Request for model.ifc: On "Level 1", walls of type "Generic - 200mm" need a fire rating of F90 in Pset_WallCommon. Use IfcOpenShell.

First a look at what the model holds.

```python
import ifcopenshell
import ifcopenshell.util.element

model = ifcopenshell.open("model.ifc")
print(model.schema)
storey = next(s for s in model.by_type("IfcBuildingStorey") if s.Name == "Level 1")
walls = [e for e in ifcopenshell.util.element.get_decomposition(storey) if e.is_a("IfcWall")]
seen = {}
for e in walls:
    element_type = ifcopenshell.util.element.get_type(e)
    key = (element_type.Name if element_type != e and element_type else None, ifcopenshell.util.element.get_pset(e, "Pset_WallCommon", "FireRating"))
    seen[key] = seen.get(key, 0) + 1
for (name, value), count in sorted(seen.items(), key=str):
    print(count, "x", name, "|", value)
```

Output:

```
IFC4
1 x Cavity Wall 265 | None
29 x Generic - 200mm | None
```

```python
import ifcopenshell
import ifcopenshell.api.pset
import ifcopenshell.util.element

model = ifcopenshell.open("model.ifc")

storey = next(s for s in model.by_type("IfcBuildingStorey") if s.Name == "Level 1")
walls = [e for e in ifcopenshell.util.element.get_decomposition(storey) if e.is_a("IfcWall")]

count = 0
for e in walls:
    element_type = ifcopenshell.util.element.get_type(e)
    if element_type in (None, e) or element_type.Name != "Generic - 200mm":
        continue
    # add_pset returns the element's existing set when there is one.
    pset = ifcopenshell.api.pset.add_pset(model, product=e, name="Pset_WallCommon")
    ifcopenshell.api.pset.edit_pset(model, pset=pset, properties={"FireRating": "F90"})
    count += 1

print(count, "walls updated")

model.write("model_rev.ifc")
```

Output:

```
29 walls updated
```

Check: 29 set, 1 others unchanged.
